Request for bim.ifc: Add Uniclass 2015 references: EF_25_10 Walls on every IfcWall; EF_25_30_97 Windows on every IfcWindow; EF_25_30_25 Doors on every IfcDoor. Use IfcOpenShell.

First a look at what the model holds.

```python
import ifcopenshell

model = ifcopenshell.open("bim.ifc")
print(model.schema)
print("classifications:", [c.Name for c in model.by_type("IfcClassification")])
for ifc_class in ("IfcDoor", "IfcRoof", "IfcStair", "IfcWall", "IfcWindow"):
    print(ifc_class, len(model.by_type(ifc_class)))
```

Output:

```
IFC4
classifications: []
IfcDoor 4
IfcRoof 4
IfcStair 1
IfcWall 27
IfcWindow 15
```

```python
import ifcopenshell
import ifcopenshell.api.classification

model = ifcopenshell.open("bim.ifc")

system = ifcopenshell.api.classification.add_classification(model, classification="Uniclass 2015")

codes = {
    "IfcWall": ("EF_25_10", "Walls"),
    "IfcWindow": ("EF_25_30_97", "Windows"),
    "IfcDoor": ("EF_25_30_25", "Doors"),
}
for ifc_class, (code, name) in codes.items():
    products = model.by_type(ifc_class)
    ifcopenshell.api.classification.add_reference(
        model, products=products, classification=system, identification=code, name=name
    )
    print(code, len(products))

model.write("bim-out.ifc")
```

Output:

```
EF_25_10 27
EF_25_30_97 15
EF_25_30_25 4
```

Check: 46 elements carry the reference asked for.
